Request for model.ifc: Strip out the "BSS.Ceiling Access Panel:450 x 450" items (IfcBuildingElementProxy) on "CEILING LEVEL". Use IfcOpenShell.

First a look at what the model holds.

```python
import ifcopenshell
import ifcopenshell.util.element

model = ifcopenshell.open("model.ifc")
print(model.schema)
storey = next(s for s in model.by_type("IfcBuildingStorey") if s.Name == "CEILING LEVEL")
proxies = [e for e in ifcopenshell.util.element.get_decomposition(storey) if e.is_a("IfcBuildingElementProxy")]
seen = {}
for e in proxies:
    element_type = ifcopenshell.util.element.get_type(e)
    name = element_type.Name if element_type not in (None, e) else None
    seen[name] = seen.get(name, 0) + 1
for name, count in sorted(seen.items(), key=str):
    print(count, "x", name)
```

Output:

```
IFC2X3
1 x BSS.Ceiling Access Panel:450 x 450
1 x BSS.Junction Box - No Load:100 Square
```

```python
import ifcopenshell
import ifcopenshell.api.root
import ifcopenshell.util.element

model = ifcopenshell.open("model.ifc")

storey = next(s for s in model.by_type("IfcBuildingStorey") if s.Name == "CEILING LEVEL")
proxies = [e for e in ifcopenshell.util.element.get_decomposition(storey) if e.is_a("IfcBuildingElementProxy")]
targets = [e for e in proxies if (t := ifcopenshell.util.element.get_type(e)) not in (None, e) and t.Name == "BSS.Ceiling Access Panel:450 x 450"]

for e in targets:
    ifcopenshell.api.root.remove_product(model, product=e)
print(len(targets), "removed")

model.write("model_v2.ifc")
```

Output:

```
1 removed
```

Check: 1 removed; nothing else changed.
